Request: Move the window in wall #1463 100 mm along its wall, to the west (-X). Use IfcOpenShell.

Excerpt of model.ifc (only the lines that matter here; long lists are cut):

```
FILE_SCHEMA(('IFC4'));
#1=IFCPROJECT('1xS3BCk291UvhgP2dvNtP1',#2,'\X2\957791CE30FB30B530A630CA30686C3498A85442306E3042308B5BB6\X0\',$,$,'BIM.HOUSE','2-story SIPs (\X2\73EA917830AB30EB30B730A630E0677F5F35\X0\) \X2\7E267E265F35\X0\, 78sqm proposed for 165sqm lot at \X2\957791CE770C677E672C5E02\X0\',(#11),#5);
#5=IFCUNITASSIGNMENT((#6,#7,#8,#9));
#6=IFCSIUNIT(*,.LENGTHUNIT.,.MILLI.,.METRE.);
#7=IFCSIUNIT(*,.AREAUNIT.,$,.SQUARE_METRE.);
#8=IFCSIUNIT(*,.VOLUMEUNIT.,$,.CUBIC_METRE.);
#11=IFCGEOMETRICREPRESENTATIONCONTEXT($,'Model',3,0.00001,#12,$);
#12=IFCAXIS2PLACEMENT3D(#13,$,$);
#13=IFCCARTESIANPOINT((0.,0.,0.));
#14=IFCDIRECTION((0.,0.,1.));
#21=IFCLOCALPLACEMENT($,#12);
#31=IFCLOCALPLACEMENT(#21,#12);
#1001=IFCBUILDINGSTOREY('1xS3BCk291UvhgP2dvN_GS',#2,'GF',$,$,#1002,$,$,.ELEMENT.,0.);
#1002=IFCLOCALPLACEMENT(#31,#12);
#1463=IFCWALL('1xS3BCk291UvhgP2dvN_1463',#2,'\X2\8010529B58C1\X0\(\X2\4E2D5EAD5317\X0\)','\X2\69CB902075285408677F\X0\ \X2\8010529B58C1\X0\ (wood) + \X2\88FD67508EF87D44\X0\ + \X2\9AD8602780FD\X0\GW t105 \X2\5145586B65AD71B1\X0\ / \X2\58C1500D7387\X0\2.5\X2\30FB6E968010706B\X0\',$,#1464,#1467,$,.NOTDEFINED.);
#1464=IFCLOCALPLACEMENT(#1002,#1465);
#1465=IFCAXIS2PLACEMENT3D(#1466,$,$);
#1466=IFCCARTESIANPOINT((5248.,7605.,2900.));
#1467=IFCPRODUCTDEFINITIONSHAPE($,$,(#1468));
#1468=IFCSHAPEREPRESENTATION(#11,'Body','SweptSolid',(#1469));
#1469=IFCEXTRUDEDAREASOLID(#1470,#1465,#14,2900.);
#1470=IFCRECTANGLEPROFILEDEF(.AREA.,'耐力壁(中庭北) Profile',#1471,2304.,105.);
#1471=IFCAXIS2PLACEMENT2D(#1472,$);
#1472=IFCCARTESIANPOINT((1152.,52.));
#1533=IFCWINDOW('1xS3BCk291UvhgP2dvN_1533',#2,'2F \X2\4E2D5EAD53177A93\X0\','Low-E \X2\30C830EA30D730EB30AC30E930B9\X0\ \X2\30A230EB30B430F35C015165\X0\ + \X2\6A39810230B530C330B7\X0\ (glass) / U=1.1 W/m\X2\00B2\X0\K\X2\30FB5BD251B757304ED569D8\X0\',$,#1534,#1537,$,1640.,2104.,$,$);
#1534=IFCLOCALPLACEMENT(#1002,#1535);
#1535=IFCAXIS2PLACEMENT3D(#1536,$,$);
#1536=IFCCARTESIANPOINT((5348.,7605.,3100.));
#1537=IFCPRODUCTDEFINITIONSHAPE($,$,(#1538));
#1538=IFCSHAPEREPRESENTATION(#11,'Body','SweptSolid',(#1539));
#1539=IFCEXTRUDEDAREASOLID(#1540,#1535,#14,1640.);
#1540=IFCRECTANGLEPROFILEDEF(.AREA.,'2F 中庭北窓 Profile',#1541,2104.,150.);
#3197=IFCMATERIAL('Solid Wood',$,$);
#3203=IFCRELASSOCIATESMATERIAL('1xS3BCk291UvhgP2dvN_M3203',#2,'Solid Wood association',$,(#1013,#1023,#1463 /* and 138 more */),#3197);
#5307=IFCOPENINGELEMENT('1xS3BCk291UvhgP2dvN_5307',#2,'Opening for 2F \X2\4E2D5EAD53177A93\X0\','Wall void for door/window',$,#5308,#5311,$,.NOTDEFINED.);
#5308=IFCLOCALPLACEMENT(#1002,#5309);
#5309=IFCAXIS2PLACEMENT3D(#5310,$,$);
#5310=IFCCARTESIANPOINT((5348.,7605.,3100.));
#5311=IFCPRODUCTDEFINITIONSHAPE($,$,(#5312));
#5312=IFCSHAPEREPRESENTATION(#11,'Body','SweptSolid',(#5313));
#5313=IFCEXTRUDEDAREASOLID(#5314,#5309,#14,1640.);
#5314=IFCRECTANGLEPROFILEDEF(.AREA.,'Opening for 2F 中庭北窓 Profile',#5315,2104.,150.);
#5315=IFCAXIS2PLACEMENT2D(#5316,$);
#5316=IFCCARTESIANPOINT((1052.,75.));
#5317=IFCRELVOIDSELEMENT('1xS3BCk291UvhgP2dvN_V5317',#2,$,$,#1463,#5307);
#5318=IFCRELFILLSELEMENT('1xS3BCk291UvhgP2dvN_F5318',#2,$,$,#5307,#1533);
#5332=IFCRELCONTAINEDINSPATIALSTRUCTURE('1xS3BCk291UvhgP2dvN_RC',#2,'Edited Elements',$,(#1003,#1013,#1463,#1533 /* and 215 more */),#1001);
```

```python
import ifcopenshell
import ifcopenshell.api.geometry
import ifcopenshell.util.placement

model = ifcopenshell.open("model.ifc")

window = model.by_guid("1xS3BCk291UvhgP2dvN_1533")
opening = window.FillsVoids[0].RelatingOpeningElement
wall = opening.VoidsElements[0].RelatingBuildingElement

wall_matrix = ifcopenshell.util.placement.get_local_placement(wall.ObjectPlacement)
shift = wall_matrix[:3, 0] * -100.0
before = ifcopenshell.util.placement.get_local_placement(window.ObjectPlacement)[:3, 3].copy()

# The window is not placed relative to its opening, so move both.
for product in (opening, window):
    matrix = ifcopenshell.util.placement.get_local_placement(product.ObjectPlacement)
    matrix[:3, 3] += shift
    ifcopenshell.api.geometry.edit_object_placement(model, product=product, matrix=matrix, is_si=False)

after = ifcopenshell.util.placement.get_local_placement(window.ObjectPlacement)[:3, 3]
print("window moved by", (after - before).round(3) + 0.0)

model.write("model_updated.ifc")
```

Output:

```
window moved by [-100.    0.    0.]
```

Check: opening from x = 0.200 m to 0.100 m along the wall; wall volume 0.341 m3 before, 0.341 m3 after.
